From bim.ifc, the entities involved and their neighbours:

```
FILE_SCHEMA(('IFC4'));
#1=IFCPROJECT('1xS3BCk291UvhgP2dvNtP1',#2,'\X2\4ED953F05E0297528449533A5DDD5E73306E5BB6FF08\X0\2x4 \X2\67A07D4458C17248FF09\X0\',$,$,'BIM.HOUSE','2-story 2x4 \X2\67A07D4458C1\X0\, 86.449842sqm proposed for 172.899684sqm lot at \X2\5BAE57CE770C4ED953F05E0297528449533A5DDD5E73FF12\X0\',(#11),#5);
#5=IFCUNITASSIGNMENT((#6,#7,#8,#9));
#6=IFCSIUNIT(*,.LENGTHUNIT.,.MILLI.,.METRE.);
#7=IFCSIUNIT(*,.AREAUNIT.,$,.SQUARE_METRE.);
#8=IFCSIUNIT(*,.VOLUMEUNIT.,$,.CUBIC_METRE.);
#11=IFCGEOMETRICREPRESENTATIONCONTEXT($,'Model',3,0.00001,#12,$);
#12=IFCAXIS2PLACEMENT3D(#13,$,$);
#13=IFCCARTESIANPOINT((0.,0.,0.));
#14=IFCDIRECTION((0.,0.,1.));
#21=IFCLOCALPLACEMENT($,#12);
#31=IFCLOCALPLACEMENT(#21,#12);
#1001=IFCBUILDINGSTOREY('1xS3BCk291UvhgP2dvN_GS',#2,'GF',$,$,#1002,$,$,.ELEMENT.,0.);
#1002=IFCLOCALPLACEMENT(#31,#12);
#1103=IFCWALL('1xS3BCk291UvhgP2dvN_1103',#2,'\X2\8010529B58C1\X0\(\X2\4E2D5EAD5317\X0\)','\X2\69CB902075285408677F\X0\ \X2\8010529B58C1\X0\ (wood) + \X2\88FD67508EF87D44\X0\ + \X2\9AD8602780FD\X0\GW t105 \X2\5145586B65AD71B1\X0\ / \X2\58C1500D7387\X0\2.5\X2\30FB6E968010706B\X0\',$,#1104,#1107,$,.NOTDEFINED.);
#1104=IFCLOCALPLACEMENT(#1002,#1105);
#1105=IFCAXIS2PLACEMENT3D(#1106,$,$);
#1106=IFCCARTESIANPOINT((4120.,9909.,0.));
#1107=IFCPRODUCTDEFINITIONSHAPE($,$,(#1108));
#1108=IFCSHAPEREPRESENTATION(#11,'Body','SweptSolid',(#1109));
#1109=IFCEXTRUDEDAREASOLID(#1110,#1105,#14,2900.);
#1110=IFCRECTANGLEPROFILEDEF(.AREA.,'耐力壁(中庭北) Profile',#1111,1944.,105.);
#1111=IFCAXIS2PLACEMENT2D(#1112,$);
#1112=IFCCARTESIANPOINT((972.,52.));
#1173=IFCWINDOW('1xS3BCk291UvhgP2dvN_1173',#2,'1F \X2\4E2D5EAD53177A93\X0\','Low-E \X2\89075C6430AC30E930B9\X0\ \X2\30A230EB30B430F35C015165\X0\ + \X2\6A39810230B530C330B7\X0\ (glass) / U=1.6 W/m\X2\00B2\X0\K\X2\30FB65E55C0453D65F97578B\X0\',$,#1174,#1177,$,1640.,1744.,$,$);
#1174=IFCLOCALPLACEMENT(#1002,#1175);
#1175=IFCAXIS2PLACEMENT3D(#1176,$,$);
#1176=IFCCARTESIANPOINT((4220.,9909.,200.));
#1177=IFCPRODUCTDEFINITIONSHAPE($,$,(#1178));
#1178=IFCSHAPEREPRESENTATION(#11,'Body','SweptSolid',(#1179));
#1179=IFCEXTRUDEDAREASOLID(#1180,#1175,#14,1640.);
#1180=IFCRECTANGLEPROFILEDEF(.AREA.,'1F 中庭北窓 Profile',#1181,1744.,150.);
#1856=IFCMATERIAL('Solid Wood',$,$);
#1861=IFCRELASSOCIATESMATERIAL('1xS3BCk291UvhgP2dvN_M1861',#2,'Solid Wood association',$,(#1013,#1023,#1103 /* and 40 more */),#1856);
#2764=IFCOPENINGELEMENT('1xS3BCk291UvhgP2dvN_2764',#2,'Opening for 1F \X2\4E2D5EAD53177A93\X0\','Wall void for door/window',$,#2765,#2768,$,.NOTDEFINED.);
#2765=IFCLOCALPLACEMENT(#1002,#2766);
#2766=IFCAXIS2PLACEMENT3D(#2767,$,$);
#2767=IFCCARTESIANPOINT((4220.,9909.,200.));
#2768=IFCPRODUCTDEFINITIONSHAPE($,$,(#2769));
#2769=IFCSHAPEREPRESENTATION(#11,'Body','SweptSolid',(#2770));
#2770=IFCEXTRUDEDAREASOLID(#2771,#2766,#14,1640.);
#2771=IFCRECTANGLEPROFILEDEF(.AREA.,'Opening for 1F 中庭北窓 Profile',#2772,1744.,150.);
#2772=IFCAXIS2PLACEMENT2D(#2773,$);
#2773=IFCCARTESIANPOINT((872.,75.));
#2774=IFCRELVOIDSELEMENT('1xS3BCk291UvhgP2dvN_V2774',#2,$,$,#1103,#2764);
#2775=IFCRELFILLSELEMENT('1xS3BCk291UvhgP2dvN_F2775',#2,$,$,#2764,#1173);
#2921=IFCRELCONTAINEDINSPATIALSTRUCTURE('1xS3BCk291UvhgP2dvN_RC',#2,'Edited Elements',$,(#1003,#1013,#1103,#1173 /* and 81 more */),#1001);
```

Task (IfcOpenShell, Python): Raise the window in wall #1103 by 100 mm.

```python
import numpy as np
import ifcopenshell
import ifcopenshell.api.geometry
import ifcopenshell.util.placement
import ifcopenshell.util.unit

model = ifcopenshell.open("bim.ifc")
unit_scale = ifcopenshell.util.unit.calculate_unit_scale(model)

window = model.by_guid("1xS3BCk291UvhgP2dvN_1173")
opening = window.FillsVoids[0].RelatingOpeningElement
dz = 100.0

shift = np.array([0.0, 0.0, dz])
# The window is not placed relative to its opening, so move both.
for product in (opening, window):
    matrix = ifcopenshell.util.placement.get_local_placement(product.ObjectPlacement)
    matrix[:3, 3] += shift
    ifcopenshell.api.geometry.edit_object_placement(model, product=product, matrix=matrix, is_si=False)

print(f"moved by {dz * unit_scale:+.3f} m")

model.write("bim_updated.ifc")
```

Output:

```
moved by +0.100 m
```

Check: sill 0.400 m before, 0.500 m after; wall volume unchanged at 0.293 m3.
